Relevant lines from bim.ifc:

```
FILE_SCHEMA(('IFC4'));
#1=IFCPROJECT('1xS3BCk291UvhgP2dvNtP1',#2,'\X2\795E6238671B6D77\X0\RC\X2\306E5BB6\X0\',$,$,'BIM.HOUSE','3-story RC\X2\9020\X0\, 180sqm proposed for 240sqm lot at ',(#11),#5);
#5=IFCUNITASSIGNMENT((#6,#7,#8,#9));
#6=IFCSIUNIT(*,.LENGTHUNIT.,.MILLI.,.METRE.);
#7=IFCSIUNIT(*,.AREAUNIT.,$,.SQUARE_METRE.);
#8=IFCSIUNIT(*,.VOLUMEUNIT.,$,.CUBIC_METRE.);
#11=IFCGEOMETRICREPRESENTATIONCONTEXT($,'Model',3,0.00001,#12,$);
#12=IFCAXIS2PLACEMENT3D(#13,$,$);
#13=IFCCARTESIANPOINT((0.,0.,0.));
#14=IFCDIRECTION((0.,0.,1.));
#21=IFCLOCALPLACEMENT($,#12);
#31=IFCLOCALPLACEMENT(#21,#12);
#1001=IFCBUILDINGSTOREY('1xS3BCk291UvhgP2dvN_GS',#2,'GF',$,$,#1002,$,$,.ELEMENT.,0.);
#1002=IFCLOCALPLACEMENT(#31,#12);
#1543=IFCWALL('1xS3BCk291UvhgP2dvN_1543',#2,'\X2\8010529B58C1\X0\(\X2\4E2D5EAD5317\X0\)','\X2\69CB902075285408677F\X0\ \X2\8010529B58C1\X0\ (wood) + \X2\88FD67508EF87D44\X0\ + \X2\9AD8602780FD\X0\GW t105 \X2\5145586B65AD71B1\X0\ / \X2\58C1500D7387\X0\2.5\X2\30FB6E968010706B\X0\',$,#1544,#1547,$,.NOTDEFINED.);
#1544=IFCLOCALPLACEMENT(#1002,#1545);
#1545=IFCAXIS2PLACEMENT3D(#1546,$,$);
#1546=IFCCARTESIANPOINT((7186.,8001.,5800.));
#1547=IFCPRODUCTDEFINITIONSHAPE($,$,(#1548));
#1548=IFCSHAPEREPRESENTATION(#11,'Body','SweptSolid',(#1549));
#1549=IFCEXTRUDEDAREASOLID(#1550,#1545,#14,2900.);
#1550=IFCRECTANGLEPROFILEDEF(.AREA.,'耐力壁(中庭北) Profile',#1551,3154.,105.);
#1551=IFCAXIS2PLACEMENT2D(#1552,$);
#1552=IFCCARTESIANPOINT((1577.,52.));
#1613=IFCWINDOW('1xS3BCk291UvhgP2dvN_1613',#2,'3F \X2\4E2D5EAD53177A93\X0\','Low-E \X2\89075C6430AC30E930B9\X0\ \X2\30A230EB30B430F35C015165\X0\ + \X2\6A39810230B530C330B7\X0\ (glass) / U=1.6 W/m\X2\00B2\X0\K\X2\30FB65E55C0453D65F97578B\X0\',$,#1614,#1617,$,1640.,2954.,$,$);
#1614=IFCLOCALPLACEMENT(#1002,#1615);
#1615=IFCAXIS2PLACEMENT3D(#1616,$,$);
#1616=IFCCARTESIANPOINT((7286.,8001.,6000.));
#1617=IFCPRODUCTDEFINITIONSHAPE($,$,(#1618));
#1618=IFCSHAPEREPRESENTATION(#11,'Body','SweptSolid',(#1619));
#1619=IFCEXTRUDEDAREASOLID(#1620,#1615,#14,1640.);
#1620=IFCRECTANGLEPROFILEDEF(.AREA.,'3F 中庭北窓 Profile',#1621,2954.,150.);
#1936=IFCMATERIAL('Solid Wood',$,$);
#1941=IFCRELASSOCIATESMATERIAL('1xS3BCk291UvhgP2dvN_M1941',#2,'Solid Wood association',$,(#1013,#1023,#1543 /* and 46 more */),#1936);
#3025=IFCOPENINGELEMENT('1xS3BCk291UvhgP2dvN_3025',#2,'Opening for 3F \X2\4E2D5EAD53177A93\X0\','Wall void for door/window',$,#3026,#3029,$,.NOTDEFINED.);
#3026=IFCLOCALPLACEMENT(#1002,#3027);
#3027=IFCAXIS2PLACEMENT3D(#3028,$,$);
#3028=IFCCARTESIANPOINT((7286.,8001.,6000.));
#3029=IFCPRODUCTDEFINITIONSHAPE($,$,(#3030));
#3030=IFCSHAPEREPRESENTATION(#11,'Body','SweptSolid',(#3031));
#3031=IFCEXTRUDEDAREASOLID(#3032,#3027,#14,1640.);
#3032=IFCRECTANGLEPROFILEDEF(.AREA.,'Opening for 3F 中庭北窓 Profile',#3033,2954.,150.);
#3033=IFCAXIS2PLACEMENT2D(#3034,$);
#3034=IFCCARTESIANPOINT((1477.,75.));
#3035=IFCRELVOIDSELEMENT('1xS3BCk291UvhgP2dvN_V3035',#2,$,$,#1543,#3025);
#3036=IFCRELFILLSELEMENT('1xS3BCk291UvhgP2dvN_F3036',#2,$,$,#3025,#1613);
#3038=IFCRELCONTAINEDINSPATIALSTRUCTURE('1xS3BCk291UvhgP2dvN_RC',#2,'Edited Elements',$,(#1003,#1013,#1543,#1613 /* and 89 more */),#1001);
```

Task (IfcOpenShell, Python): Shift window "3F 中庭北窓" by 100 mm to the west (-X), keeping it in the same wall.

```python
import ifcopenshell
import ifcopenshell.api.geometry
import ifcopenshell.util.placement
import ifcopenshell.util.unit

model = ifcopenshell.open("bim.ifc")
unit_scale = ifcopenshell.util.unit.calculate_unit_scale(model)

window = model.by_id(1613)
opening = window.FillsVoids[0].RelatingOpeningElement
wall = opening.VoidsElements[0].RelatingBuildingElement

wall_matrix = ifcopenshell.util.placement.get_local_placement(wall.ObjectPlacement)
shift = wall_matrix[:3, 0] * -0.1 / unit_scale
before = ifcopenshell.util.placement.get_local_placement(window.ObjectPlacement)[:3, 3].copy()

# The window is not placed relative to its opening, so move both.
for product in (opening, window):
    matrix = ifcopenshell.util.placement.get_local_placement(product.ObjectPlacement)
    matrix[:3, 3] += shift
    ifcopenshell.api.geometry.edit_object_placement(model, product=product, matrix=matrix, is_si=False)

after = ifcopenshell.util.placement.get_local_placement(window.ObjectPlacement)[:3, 3]
print("window moved by", (after - before).round(3) + 0.0)

model.write("bim_rev.ifc")
```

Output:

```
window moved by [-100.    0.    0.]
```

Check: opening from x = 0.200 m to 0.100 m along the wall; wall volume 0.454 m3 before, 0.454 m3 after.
